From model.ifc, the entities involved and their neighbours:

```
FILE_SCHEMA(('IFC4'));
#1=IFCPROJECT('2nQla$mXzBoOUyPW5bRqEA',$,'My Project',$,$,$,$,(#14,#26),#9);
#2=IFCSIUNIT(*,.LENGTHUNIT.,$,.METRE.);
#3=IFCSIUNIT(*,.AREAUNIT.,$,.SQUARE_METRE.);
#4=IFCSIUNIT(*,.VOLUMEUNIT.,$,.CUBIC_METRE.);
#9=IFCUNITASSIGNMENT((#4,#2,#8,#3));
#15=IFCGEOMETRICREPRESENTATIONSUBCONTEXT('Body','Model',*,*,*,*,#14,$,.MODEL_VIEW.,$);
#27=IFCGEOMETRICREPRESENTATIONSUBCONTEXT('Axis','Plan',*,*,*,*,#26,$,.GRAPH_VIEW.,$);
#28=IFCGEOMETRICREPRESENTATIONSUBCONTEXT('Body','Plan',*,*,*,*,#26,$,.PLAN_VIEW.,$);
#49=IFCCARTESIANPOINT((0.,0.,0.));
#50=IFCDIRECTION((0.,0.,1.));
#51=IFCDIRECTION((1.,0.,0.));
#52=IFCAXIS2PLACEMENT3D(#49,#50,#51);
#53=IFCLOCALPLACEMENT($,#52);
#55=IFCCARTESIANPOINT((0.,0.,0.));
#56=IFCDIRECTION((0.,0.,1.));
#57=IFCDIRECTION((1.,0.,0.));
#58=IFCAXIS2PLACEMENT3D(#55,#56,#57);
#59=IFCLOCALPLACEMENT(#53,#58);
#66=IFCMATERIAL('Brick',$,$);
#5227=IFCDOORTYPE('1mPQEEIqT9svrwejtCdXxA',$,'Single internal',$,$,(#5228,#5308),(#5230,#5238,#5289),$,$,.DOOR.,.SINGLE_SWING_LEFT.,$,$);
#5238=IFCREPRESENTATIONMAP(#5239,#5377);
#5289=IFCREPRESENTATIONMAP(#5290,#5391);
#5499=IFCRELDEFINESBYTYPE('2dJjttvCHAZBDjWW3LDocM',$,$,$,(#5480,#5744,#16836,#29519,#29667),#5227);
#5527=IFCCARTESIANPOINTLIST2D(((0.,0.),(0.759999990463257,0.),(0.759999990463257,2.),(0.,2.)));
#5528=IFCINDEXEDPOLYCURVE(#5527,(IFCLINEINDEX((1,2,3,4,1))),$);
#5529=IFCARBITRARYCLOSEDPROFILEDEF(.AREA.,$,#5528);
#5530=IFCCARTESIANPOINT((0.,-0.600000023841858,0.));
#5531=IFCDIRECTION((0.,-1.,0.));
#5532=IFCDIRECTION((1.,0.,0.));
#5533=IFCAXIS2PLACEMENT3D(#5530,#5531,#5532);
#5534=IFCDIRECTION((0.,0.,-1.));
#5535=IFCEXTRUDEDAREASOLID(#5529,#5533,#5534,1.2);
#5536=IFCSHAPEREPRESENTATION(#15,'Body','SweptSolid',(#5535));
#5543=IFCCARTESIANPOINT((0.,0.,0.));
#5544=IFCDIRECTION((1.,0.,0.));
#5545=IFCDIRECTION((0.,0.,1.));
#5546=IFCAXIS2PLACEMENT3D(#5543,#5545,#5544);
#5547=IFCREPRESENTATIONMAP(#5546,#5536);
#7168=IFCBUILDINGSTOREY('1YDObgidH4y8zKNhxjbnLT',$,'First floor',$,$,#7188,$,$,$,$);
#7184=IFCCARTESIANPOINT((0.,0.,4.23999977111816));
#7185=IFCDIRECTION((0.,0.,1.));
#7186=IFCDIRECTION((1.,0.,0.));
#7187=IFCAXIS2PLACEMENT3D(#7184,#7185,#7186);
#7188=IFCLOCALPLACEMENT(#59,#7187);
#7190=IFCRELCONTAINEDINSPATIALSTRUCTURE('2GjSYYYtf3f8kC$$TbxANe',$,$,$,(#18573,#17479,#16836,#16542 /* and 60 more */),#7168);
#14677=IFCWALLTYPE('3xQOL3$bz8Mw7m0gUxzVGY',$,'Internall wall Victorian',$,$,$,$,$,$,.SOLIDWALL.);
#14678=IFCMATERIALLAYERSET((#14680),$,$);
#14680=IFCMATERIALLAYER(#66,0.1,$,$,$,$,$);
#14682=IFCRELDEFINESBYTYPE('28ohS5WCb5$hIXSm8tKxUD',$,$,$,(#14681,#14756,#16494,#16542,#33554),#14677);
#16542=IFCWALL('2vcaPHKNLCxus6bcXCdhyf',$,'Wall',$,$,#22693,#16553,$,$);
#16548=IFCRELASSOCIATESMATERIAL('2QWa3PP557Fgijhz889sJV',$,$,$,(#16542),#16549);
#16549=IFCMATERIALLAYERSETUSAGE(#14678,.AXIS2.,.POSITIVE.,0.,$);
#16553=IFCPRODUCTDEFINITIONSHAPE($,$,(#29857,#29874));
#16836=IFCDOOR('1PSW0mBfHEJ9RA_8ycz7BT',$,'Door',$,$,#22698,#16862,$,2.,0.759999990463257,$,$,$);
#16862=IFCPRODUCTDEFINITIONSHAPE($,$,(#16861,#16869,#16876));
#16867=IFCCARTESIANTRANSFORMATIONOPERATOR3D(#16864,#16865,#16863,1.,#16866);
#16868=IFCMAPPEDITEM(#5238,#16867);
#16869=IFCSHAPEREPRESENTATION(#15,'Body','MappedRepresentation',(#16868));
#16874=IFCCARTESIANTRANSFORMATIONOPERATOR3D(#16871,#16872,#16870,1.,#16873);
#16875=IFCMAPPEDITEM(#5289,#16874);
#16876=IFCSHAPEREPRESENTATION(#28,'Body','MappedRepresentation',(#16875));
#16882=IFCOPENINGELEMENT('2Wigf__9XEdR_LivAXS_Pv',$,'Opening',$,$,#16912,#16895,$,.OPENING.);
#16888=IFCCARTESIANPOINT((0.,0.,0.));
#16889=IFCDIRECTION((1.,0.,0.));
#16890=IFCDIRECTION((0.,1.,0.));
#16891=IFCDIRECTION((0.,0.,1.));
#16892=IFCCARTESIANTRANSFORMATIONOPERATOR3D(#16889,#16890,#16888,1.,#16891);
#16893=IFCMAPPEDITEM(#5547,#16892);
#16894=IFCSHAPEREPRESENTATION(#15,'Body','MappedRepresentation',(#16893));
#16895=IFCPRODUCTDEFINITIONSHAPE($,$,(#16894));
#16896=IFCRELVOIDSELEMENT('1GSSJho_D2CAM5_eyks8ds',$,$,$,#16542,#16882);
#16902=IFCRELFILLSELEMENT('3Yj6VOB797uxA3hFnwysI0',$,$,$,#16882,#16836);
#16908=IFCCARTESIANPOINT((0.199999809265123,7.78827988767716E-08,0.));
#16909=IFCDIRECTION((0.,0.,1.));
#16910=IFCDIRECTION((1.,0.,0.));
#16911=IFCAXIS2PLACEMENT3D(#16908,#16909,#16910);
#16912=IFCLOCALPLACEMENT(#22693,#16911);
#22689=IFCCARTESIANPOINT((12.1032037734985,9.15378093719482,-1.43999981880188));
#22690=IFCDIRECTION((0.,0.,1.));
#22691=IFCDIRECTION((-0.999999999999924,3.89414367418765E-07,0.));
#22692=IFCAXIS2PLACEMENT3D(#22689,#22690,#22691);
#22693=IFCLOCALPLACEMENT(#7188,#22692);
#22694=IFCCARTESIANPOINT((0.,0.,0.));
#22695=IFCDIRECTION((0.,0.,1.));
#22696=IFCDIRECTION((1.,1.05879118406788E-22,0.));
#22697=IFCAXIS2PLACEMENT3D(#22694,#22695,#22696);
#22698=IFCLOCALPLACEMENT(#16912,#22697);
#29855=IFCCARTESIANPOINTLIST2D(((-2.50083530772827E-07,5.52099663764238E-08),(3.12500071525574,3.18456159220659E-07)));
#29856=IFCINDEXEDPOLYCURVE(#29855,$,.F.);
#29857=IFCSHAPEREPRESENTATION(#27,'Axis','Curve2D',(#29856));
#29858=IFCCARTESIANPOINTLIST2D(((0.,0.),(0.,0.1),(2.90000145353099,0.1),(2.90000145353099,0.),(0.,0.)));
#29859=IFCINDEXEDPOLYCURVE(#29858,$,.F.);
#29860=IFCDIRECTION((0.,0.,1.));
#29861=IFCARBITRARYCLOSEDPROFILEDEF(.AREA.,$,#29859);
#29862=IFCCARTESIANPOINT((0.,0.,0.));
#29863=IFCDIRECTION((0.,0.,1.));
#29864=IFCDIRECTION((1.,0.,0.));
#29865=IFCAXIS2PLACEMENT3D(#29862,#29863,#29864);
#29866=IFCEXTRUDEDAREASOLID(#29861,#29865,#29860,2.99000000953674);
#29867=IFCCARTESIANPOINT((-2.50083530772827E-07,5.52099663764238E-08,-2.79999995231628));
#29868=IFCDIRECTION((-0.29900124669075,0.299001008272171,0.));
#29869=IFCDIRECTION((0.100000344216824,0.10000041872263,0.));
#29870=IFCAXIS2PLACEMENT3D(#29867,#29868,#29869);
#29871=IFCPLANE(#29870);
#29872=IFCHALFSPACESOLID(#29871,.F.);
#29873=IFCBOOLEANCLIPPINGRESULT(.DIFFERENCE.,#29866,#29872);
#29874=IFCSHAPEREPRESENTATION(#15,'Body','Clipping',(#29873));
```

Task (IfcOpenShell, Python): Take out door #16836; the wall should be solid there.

```python
import ifcopenshell
import ifcopenshell.api.feature
import ifcopenshell.api.root
import ifcopenshell.geom
import ifcopenshell.util.shape

model = ifcopenshell.open("model.ifc")
settings = ifcopenshell.geom.settings()


def volume(element):
    """Net volume in cubic metres, openings subtracted."""
    shape = ifcopenshell.geom.create_shape(settings, element)
    return ifcopenshell.util.shape.get_volume(shape.geometry)


door = model.by_guid("1PSW0mBfHEJ9RA_8ycz7BT")
opening = door.FillsVoids[0].RelatingOpeningElement
wall = opening.VoidsElements[0].RelatingBuildingElement
before = volume(wall)

ifcopenshell.api.root.remove_product(model, product=door)
ifcopenshell.api.feature.remove_feature(model, feature=opening)

after = volume(wall)

print(f"wall volume {before:.3f} -> {after:.3f} m3")

model.write("model_edited.ifc")
```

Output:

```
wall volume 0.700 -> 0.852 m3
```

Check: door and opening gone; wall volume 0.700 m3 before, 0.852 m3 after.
